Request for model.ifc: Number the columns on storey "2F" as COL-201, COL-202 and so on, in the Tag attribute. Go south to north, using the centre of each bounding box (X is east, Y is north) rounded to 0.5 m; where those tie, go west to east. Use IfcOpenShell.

First a look at what the model holds.

```python
import ifcopenshell
import ifcopenshell.util.element
import ifcopenshell.util.placement

model = ifcopenshell.open("model.ifc")
print(model.schema)
storey = next(s for s in model.by_type("IfcBuildingStorey") if s.Name == "2F")
columns = [e for e in ifcopenshell.util.element.get_decomposition(storey) if e.is_a("IfcColumn")]
for e in sorted(columns, key=lambda e: e.id()):
    origin = ifcopenshell.util.placement.get_local_placement(e.ObjectPlacement)[:3, 3]
    print(e.id(), e.Tag, e.Name, origin.round(2) + 0.0, sep=" | ")
```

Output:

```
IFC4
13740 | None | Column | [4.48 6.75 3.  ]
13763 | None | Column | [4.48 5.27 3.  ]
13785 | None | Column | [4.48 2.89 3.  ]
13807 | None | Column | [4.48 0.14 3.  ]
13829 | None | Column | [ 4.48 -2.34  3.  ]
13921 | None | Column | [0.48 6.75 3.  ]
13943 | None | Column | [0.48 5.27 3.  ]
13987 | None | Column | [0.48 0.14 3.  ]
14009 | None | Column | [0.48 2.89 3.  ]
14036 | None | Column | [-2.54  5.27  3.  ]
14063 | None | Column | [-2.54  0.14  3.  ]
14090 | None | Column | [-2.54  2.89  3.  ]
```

```python
import ifcopenshell
import ifcopenshell.geom
import ifcopenshell.util.element
import ifcopenshell.util.shape

model = ifcopenshell.open("model.ifc")
settings = ifcopenshell.geom.settings()
settings.set("use-world-coords", True)


def centre(element):
    shape = ifcopenshell.geom.create_shape(settings, element)
    return ifcopenshell.util.shape.get_bbox_centroid(shape.geometry)


storey = next(s for s in model.by_type("IfcBuildingStorey") if s.Name == "2F")
columns = [e for e in ifcopenshell.util.element.get_decomposition(storey) if e.is_a("IfcColumn")]

# Insertion points can sit at a corner or the storey origin, so sort by the geometry (in metres).
centres = {e: centre(e) for e in columns}
columns.sort(key=lambda e: (round(centres[e][1] / 0.5), centres[e][0]))

for i, e in enumerate(columns, start=1):
    number = f"COL-2{i:02d}"
    e.Tag = number
    print(e.id(), number)

model.write("model_v2.ifc")
```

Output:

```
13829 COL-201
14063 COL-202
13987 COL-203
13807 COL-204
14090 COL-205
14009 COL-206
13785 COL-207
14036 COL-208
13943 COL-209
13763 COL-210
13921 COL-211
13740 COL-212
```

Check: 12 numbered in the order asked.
